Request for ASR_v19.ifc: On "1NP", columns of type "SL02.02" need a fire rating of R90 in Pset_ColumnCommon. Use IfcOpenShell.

First a look at what the model holds.

```python
import ifcopenshell
import ifcopenshell.util.element

model = ifcopenshell.open("ASR_v19.ifc")
print(model.schema)
storey = next(s for s in model.by_type("IfcBuildingStorey") if s.Name == "1NP")
columns = [e for e in ifcopenshell.util.element.get_decomposition(storey) if e.is_a("IfcColumn")]
seen = {}
for e in columns:
    element_type = ifcopenshell.util.element.get_type(e)
    key = (element_type.Name if element_type != e and element_type else None, ifcopenshell.util.element.get_pset(e, "Pset_ColumnCommon", "FireRating"))
    seen[key] = seen.get(key, 0) + 1
for (name, value), count in sorted(seen.items(), key=str):
    print(count, "x", name, "|", value)
```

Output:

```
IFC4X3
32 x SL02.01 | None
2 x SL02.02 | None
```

```python
import ifcopenshell
import ifcopenshell.api.pset
import ifcopenshell.util.element

model = ifcopenshell.open("ASR_v19.ifc")

storey = next(s for s in model.by_type("IfcBuildingStorey") if s.Name == "1NP")
columns = [e for e in ifcopenshell.util.element.get_decomposition(storey) if e.is_a("IfcColumn")]

count = 0
for e in columns:
    element_type = ifcopenshell.util.element.get_type(e)
    if element_type in (None, e) or element_type.Name != "SL02.02":
        continue
    # add_pset returns the element's existing set when there is one.
    pset = ifcopenshell.api.pset.add_pset(model, product=e, name="Pset_ColumnCommon")
    ifcopenshell.api.pset.edit_pset(model, pset=pset, properties={"FireRating": "R90"})
    count += 1

print(count, "columns updated")

model.write("ASR_v19-out.ifc")
```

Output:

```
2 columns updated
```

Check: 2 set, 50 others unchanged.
